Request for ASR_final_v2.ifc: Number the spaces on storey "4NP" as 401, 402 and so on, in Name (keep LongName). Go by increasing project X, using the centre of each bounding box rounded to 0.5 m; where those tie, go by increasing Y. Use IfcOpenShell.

First a look at what the model holds.

```python
import ifcopenshell
import ifcopenshell.util.element
import ifcopenshell.util.placement

model = ifcopenshell.open("ASR_final_v2.ifc")
print(model.schema)
storey = next(s for s in model.by_type("IfcBuildingStorey") if s.Name == "4NP")
spaces = [e for e in ifcopenshell.util.element.get_decomposition(storey) if e.is_a("IfcSpace")]
for e in sorted(spaces, key=lambda e: e.id()):
    origin = ifcopenshell.util.placement.get_local_placement(e.ObjectPlacement)[:3, 3]
    print(e.id(), e.Name, e.LongName, origin.round(2) + 0.0, sep=" | ")
```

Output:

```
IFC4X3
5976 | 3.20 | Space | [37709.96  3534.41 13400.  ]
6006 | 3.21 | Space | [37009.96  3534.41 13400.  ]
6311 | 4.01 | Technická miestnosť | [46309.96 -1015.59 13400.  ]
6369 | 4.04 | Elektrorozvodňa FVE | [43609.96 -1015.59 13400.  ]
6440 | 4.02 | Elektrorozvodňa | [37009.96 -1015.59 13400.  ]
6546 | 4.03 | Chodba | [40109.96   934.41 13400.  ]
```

```python
import ifcopenshell
import ifcopenshell.geom
import ifcopenshell.util.element
import ifcopenshell.util.shape

model = ifcopenshell.open("ASR_final_v2.ifc")
settings = ifcopenshell.geom.settings()
settings.set("use-world-coords", True)


def centre(element):
    shape = ifcopenshell.geom.create_shape(settings, element)
    return ifcopenshell.util.shape.get_bbox_centroid(shape.geometry)


storey = next(s for s in model.by_type("IfcBuildingStorey") if s.Name == "4NP")
spaces = [e for e in ifcopenshell.util.element.get_decomposition(storey) if e.is_a("IfcSpace")]

# Insertion points can sit at a corner or the storey origin, so sort by the geometry (in metres).
centres = {e: centre(e) for e in spaces}
spaces.sort(key=lambda e: (round(centres[e][0] / 0.5), centres[e][1]))

for i, e in enumerate(spaces, start=1):
    number = f"4{i:02d}"
    e.Name = number
    print(e.id(), number)

model.write("ASR_final_v2_edited.ifc")
```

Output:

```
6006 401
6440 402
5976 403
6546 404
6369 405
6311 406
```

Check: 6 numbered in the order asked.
